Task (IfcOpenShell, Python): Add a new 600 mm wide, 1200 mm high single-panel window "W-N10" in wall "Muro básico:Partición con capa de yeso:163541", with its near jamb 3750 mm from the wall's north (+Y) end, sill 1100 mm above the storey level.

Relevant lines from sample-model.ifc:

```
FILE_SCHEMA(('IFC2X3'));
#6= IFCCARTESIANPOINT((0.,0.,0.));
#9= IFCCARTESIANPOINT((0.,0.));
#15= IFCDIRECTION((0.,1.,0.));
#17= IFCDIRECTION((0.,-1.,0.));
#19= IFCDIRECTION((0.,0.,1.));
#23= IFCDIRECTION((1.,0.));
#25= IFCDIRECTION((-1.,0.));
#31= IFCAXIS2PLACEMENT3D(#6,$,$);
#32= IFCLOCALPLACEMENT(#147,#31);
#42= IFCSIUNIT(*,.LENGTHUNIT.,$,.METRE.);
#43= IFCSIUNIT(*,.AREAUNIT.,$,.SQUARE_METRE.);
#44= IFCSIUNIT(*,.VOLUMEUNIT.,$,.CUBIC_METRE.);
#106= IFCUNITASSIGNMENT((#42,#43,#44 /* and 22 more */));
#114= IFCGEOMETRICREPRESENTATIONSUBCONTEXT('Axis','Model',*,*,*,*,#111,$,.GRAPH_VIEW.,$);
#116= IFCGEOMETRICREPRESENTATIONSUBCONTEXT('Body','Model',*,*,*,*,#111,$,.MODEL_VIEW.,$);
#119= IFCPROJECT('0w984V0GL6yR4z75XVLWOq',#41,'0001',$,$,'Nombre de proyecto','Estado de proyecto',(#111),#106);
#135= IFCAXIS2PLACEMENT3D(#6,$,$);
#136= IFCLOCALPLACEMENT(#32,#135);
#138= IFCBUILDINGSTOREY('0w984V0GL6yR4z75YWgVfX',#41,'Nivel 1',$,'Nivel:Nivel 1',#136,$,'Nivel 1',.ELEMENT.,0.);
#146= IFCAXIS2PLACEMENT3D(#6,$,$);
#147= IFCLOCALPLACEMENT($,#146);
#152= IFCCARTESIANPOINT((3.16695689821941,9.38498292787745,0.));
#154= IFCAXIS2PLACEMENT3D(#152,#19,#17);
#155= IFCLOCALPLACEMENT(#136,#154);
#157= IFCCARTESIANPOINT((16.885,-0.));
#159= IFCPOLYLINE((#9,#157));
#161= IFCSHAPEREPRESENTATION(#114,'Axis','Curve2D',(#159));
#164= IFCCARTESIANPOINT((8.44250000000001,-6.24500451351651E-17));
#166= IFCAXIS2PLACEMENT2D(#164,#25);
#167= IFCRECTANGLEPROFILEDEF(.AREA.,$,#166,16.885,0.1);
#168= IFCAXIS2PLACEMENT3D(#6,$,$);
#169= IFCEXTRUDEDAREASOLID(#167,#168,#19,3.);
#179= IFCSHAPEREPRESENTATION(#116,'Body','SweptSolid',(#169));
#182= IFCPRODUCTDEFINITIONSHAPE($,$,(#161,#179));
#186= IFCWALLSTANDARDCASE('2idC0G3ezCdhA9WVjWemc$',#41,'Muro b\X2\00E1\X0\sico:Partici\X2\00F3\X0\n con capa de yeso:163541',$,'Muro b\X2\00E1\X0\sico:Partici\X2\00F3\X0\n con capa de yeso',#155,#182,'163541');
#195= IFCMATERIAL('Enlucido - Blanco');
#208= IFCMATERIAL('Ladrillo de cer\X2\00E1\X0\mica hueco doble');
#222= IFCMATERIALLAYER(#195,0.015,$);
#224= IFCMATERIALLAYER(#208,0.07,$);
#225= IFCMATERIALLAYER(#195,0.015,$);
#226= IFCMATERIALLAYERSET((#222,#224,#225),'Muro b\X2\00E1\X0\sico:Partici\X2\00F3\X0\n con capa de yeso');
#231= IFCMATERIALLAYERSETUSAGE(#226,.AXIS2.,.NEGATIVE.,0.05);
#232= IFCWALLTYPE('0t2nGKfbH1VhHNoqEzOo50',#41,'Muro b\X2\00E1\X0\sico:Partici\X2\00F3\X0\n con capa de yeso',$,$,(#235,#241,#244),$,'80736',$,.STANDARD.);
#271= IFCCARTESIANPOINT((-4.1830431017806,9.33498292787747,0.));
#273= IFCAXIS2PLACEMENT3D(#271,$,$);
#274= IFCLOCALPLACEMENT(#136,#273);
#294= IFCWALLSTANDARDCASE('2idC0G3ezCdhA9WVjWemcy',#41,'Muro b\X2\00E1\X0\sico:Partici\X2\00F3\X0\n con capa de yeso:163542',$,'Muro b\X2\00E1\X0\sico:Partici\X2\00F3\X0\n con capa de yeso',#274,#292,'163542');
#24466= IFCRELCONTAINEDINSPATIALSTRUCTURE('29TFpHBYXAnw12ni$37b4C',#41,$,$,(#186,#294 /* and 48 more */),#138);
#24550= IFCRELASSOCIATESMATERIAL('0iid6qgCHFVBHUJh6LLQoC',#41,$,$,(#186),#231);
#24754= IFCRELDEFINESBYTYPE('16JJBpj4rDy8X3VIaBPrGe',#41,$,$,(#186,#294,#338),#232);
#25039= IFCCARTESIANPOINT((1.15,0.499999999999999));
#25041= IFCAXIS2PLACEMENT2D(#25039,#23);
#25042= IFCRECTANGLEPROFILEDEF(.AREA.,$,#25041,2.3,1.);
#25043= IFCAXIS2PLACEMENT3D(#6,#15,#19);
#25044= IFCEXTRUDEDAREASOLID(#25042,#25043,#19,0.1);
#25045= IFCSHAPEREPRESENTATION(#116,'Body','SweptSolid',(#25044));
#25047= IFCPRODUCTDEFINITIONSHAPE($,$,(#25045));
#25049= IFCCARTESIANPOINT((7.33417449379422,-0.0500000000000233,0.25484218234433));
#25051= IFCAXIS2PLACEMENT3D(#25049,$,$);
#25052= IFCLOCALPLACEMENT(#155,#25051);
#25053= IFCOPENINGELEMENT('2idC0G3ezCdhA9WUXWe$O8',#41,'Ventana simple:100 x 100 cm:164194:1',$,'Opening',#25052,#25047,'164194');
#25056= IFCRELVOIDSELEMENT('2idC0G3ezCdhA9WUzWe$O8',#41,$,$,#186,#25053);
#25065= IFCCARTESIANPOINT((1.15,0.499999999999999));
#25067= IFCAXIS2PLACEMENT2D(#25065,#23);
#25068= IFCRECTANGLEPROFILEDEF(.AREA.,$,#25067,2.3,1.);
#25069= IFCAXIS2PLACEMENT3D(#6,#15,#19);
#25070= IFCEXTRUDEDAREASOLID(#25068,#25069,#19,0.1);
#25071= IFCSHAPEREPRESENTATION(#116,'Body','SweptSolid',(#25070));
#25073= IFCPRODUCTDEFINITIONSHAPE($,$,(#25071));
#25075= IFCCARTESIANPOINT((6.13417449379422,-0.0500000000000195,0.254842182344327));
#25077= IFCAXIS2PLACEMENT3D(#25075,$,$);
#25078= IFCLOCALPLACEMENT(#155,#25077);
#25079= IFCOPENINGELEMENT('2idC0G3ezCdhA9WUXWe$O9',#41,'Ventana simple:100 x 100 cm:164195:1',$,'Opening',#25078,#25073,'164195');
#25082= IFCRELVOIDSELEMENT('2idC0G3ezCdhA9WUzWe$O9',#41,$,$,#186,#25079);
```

```python
import numpy as np
import ifcopenshell
import ifcopenshell.api.feature
import ifcopenshell.api.geometry
import ifcopenshell.api.root
import ifcopenshell.api.spatial
import ifcopenshell.api.type
import ifcopenshell.geom
import ifcopenshell.util.element
import ifcopenshell.util.placement
import ifcopenshell.util.representation
import ifcopenshell.util.shape
import ifcopenshell.util.unit

model = ifcopenshell.open("sample-model.ifc")
unit_scale = ifcopenshell.util.unit.calculate_unit_scale(model)
settings = ifcopenshell.geom.settings()


def volume(element):
    """Net volume in cubic metres, openings subtracted."""
    shape = ifcopenshell.geom.create_shape(settings, element)
    return ifcopenshell.util.shape.get_volume(shape.geometry)


wall = model.by_id(186)
storey = ifcopenshell.util.element.get_container(wall, ifc_class="IfcBuildingStorey")
context = ifcopenshell.util.representation.get_context(model, "Model", "Body", "MODEL_VIEW")
before = volume(wall)

width, height, from_end, sill = 0.6, 1.2, 3.75, 1.1  # metres

# The wall runs along its own X axis, and the end named is its -X end.
wall_shape = ifcopenshell.geom.create_shape(settings, wall)
x, y, z = ifcopenshell.util.shape.get_vertices(wall_shape.geometry).T
start = x.min() + from_end
face, thickness = float(y.min()), float(y.max() - y.min())
wall_matrix = ifcopenshell.util.placement.get_local_placement(wall.ObjectPlacement)
level = ifcopenshell.util.placement.get_local_placement(storey.ObjectPlacement)[2, 3]


def in_wall(x, y):
    """Placement at x, y metres in the wall's axes, at sill height."""
    matrix = wall_matrix.copy()
    matrix[:, 3] = wall_matrix @ np.array([x / unit_scale, y / unit_scale, 0.0, 1.0])
    matrix[2, 3] = level + sill / unit_scale
    return matrix


# Opening: a box that overshoots both wall faces by 50 mm.
opening = ifcopenshell.api.root.create_entity(model, ifc_class="IfcOpeningElement")
box = ifcopenshell.api.geometry.add_wall_representation(
    model, context=context, length=width, height=height, thickness=thickness + 0.1
)
ifcopenshell.api.geometry.assign_representation(model, product=opening, representation=box)
ifcopenshell.api.geometry.edit_object_placement(model, product=opening, matrix=in_wall(start, face - 0.05), is_si=False)
ifcopenshell.api.feature.add_feature(model, feature=opening, element=wall)

window = ifcopenshell.api.root.create_entity(model, ifc_class="IfcWindow", name="W-N10")
window.OverallWidth, window.OverallHeight = width / unit_scale, height / unit_scale
body = ifcopenshell.api.geometry.add_window_representation(
    model,
    context=context,
    overall_width=window.OverallWidth,
    overall_height=window.OverallHeight,
    partition_type="SINGLE_PANEL",
)
ifcopenshell.api.geometry.assign_representation(model, product=window, representation=body)
ifcopenshell.api.spatial.assign_container(model, products=[window], relating_structure=storey)
fills = ifcopenshell.api.feature.add_filling(model, opening=opening, element=window)
fills.OwnerHistory = window.OwnerHistory  # required in IFC2X3

# IFC2X3 keeps the operation on the window style.
style = ifcopenshell.api.root.create_entity(model, ifc_class="IfcWindowStyle", name="W-N10")
style.OperationType, style.ConstructionType = "SINGLE_PANEL", "NOTDEFINED"
style.ParameterTakesPrecedence = style.Sizeable = False
ifcopenshell.api.type.assign_type(model, related_objects=[window], relating_type=style)

# Centre the window in the wall's thickness.
ifcopenshell.api.geometry.edit_object_placement(model, product=window, matrix=in_wall(start, face), is_si=False)
window_shape = ifcopenshell.geom.create_shape(settings, window)
depth = ifcopenshell.util.shape.get_vertices(window_shape.geometry)[:, 1]
offset = face + thickness / 2 - (depth.min() + depth.max()) / 2
ifcopenshell.api.geometry.edit_object_placement(model, product=window, matrix=in_wall(start, offset), is_si=False)

after = volume(wall)

print(f"wall volume {before:.3f} -> {after:.3f} m3")

model.write("sample-model_rev.ifc")
```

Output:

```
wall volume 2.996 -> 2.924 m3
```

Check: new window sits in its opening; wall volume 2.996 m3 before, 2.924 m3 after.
